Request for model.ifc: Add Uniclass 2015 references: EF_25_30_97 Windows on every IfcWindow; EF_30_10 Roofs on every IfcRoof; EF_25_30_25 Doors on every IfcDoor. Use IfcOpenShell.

First a look at what the model holds.

```python
import ifcopenshell

model = ifcopenshell.open("model.ifc")
print(model.schema)
print("classifications:", [c.Name for c in model.by_type("IfcClassification")])
for ifc_class in ("IfcDoor", "IfcRoof", "IfcStair", "IfcWall", "IfcWindow"):
    print(ifc_class, len(model.by_type(ifc_class)))
```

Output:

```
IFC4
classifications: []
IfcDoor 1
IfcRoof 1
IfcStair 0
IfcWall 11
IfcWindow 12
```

```python
import ifcopenshell
import ifcopenshell.api.classification

model = ifcopenshell.open("model.ifc")

system = ifcopenshell.api.classification.add_classification(model, classification="Uniclass 2015")

codes = {
    "IfcWindow": ("EF_25_30_97", "Windows"),
    "IfcRoof": ("EF_30_10", "Roofs"),
    "IfcDoor": ("EF_25_30_25", "Doors"),
}
for ifc_class, (code, name) in codes.items():
    products = model.by_type(ifc_class)
    ifcopenshell.api.classification.add_reference(
        model, products=products, classification=system, identification=code, name=name
    )
    print(code, len(products))

model.write("model_v2.ifc")
```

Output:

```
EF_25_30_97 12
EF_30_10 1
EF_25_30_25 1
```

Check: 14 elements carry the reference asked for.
